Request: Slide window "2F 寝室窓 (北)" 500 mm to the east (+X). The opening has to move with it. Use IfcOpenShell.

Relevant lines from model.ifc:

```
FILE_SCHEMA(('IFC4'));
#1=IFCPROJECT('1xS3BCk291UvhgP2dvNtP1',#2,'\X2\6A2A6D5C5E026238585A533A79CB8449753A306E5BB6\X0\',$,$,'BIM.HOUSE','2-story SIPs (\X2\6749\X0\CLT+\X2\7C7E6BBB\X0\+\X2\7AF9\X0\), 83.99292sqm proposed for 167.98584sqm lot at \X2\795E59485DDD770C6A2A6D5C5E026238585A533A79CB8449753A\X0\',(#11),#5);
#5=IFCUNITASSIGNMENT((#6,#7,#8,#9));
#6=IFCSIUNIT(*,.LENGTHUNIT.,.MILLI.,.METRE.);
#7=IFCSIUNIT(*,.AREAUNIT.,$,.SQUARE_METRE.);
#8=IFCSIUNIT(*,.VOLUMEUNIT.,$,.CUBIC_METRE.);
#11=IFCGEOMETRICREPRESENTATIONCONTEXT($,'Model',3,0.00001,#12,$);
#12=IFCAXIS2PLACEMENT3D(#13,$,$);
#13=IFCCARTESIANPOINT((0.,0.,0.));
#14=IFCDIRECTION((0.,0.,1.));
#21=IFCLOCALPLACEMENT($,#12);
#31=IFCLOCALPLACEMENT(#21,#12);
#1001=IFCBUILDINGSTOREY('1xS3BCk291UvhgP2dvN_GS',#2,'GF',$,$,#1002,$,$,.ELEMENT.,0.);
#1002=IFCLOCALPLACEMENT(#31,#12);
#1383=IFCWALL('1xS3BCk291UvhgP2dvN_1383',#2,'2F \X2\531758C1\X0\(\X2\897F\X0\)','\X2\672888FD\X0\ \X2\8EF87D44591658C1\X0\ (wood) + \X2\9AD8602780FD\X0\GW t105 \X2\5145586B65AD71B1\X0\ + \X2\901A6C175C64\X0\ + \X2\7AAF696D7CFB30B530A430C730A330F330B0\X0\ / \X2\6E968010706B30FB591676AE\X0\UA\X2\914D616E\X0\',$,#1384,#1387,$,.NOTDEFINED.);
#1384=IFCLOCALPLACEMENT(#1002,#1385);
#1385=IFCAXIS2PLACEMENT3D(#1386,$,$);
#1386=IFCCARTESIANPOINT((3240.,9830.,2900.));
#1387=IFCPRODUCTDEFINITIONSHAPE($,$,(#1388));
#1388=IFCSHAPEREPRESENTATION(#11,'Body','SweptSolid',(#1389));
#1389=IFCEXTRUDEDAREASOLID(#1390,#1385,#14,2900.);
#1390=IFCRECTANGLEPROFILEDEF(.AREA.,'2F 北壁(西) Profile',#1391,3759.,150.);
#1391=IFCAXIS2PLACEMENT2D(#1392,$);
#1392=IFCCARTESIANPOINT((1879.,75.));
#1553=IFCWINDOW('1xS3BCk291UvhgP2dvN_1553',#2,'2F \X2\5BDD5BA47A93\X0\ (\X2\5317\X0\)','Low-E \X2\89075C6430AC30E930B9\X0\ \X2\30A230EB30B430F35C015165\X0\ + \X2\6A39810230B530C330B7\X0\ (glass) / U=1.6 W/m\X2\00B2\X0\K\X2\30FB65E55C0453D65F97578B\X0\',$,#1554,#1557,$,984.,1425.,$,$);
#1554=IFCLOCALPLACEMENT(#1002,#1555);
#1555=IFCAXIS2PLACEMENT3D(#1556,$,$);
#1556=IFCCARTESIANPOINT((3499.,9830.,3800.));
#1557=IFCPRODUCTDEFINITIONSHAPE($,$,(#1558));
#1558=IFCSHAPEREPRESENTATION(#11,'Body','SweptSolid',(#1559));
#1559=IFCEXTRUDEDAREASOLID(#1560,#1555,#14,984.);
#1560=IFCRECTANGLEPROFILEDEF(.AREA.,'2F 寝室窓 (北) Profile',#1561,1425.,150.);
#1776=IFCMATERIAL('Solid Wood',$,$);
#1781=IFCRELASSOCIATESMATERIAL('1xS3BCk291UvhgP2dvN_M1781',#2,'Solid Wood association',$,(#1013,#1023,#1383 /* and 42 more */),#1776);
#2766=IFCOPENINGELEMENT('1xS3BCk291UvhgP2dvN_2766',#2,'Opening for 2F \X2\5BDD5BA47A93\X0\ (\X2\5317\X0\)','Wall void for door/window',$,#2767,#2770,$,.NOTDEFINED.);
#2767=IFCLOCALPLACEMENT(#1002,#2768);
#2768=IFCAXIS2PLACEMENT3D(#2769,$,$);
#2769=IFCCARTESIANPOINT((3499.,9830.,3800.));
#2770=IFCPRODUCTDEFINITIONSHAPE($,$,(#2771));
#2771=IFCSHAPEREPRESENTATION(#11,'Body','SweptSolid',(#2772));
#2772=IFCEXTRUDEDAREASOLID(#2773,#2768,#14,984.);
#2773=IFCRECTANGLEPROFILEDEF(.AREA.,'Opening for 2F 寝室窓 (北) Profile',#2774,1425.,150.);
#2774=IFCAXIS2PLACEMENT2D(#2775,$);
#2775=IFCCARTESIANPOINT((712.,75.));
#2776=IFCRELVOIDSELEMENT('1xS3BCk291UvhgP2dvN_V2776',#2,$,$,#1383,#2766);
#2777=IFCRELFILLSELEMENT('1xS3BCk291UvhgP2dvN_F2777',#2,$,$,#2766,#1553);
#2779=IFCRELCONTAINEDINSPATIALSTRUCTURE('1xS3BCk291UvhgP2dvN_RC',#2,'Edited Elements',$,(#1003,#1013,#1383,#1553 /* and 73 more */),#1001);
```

```python
import ifcopenshell
import ifcopenshell.api.geometry
import ifcopenshell.util.placement

model = ifcopenshell.open("model.ifc")

window = model.by_guid("1xS3BCk291UvhgP2dvN_1553")
opening = window.FillsVoids[0].RelatingOpeningElement
wall = opening.VoidsElements[0].RelatingBuildingElement

wall_matrix = ifcopenshell.util.placement.get_local_placement(wall.ObjectPlacement)
shift = wall_matrix[:3, 0] * 500.0
before = ifcopenshell.util.placement.get_local_placement(window.ObjectPlacement)[:3, 3].copy()

# The window is not placed relative to its opening, so move both.
for product in (opening, window):
    matrix = ifcopenshell.util.placement.get_local_placement(product.ObjectPlacement)
    matrix[:3, 3] += shift
    ifcopenshell.api.geometry.edit_object_placement(model, product=product, matrix=matrix, is_si=False)

after = ifcopenshell.util.placement.get_local_placement(window.ObjectPlacement)[:3, 3]
print("window moved by", (after - before).round(3) + 0.0)

model.write("model_updated.ifc")
```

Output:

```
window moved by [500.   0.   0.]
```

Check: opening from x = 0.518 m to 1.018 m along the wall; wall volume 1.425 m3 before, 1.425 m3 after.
